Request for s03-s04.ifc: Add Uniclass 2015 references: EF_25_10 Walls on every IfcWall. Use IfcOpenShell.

First a look at what the model holds.

```python
import ifcopenshell

model = ifcopenshell.open("s03-s04.ifc")
print(model.schema)
print("classifications:", [c.Name for c in model.by_type("IfcClassification")])
for ifc_class in ("IfcDoor", "IfcRoof", "IfcStair", "IfcWall", "IfcWindow"):
    print(ifc_class, len(model.by_type(ifc_class)))
```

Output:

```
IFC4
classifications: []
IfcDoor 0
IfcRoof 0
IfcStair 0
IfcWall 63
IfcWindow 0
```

```python
import ifcopenshell
import ifcopenshell.api.classification

model = ifcopenshell.open("s03-s04.ifc")

system = ifcopenshell.api.classification.add_classification(model, classification="Uniclass 2015")

codes = {
    "IfcWall": ("EF_25_10", "Walls"),
}
for ifc_class, (code, name) in codes.items():
    products = model.by_type(ifc_class)
    ifcopenshell.api.classification.add_reference(
        model, products=products, classification=system, identification=code, name=name
    )
    print(code, len(products))

model.write("s03-s04_edited.ifc")
```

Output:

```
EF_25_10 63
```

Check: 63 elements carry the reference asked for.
